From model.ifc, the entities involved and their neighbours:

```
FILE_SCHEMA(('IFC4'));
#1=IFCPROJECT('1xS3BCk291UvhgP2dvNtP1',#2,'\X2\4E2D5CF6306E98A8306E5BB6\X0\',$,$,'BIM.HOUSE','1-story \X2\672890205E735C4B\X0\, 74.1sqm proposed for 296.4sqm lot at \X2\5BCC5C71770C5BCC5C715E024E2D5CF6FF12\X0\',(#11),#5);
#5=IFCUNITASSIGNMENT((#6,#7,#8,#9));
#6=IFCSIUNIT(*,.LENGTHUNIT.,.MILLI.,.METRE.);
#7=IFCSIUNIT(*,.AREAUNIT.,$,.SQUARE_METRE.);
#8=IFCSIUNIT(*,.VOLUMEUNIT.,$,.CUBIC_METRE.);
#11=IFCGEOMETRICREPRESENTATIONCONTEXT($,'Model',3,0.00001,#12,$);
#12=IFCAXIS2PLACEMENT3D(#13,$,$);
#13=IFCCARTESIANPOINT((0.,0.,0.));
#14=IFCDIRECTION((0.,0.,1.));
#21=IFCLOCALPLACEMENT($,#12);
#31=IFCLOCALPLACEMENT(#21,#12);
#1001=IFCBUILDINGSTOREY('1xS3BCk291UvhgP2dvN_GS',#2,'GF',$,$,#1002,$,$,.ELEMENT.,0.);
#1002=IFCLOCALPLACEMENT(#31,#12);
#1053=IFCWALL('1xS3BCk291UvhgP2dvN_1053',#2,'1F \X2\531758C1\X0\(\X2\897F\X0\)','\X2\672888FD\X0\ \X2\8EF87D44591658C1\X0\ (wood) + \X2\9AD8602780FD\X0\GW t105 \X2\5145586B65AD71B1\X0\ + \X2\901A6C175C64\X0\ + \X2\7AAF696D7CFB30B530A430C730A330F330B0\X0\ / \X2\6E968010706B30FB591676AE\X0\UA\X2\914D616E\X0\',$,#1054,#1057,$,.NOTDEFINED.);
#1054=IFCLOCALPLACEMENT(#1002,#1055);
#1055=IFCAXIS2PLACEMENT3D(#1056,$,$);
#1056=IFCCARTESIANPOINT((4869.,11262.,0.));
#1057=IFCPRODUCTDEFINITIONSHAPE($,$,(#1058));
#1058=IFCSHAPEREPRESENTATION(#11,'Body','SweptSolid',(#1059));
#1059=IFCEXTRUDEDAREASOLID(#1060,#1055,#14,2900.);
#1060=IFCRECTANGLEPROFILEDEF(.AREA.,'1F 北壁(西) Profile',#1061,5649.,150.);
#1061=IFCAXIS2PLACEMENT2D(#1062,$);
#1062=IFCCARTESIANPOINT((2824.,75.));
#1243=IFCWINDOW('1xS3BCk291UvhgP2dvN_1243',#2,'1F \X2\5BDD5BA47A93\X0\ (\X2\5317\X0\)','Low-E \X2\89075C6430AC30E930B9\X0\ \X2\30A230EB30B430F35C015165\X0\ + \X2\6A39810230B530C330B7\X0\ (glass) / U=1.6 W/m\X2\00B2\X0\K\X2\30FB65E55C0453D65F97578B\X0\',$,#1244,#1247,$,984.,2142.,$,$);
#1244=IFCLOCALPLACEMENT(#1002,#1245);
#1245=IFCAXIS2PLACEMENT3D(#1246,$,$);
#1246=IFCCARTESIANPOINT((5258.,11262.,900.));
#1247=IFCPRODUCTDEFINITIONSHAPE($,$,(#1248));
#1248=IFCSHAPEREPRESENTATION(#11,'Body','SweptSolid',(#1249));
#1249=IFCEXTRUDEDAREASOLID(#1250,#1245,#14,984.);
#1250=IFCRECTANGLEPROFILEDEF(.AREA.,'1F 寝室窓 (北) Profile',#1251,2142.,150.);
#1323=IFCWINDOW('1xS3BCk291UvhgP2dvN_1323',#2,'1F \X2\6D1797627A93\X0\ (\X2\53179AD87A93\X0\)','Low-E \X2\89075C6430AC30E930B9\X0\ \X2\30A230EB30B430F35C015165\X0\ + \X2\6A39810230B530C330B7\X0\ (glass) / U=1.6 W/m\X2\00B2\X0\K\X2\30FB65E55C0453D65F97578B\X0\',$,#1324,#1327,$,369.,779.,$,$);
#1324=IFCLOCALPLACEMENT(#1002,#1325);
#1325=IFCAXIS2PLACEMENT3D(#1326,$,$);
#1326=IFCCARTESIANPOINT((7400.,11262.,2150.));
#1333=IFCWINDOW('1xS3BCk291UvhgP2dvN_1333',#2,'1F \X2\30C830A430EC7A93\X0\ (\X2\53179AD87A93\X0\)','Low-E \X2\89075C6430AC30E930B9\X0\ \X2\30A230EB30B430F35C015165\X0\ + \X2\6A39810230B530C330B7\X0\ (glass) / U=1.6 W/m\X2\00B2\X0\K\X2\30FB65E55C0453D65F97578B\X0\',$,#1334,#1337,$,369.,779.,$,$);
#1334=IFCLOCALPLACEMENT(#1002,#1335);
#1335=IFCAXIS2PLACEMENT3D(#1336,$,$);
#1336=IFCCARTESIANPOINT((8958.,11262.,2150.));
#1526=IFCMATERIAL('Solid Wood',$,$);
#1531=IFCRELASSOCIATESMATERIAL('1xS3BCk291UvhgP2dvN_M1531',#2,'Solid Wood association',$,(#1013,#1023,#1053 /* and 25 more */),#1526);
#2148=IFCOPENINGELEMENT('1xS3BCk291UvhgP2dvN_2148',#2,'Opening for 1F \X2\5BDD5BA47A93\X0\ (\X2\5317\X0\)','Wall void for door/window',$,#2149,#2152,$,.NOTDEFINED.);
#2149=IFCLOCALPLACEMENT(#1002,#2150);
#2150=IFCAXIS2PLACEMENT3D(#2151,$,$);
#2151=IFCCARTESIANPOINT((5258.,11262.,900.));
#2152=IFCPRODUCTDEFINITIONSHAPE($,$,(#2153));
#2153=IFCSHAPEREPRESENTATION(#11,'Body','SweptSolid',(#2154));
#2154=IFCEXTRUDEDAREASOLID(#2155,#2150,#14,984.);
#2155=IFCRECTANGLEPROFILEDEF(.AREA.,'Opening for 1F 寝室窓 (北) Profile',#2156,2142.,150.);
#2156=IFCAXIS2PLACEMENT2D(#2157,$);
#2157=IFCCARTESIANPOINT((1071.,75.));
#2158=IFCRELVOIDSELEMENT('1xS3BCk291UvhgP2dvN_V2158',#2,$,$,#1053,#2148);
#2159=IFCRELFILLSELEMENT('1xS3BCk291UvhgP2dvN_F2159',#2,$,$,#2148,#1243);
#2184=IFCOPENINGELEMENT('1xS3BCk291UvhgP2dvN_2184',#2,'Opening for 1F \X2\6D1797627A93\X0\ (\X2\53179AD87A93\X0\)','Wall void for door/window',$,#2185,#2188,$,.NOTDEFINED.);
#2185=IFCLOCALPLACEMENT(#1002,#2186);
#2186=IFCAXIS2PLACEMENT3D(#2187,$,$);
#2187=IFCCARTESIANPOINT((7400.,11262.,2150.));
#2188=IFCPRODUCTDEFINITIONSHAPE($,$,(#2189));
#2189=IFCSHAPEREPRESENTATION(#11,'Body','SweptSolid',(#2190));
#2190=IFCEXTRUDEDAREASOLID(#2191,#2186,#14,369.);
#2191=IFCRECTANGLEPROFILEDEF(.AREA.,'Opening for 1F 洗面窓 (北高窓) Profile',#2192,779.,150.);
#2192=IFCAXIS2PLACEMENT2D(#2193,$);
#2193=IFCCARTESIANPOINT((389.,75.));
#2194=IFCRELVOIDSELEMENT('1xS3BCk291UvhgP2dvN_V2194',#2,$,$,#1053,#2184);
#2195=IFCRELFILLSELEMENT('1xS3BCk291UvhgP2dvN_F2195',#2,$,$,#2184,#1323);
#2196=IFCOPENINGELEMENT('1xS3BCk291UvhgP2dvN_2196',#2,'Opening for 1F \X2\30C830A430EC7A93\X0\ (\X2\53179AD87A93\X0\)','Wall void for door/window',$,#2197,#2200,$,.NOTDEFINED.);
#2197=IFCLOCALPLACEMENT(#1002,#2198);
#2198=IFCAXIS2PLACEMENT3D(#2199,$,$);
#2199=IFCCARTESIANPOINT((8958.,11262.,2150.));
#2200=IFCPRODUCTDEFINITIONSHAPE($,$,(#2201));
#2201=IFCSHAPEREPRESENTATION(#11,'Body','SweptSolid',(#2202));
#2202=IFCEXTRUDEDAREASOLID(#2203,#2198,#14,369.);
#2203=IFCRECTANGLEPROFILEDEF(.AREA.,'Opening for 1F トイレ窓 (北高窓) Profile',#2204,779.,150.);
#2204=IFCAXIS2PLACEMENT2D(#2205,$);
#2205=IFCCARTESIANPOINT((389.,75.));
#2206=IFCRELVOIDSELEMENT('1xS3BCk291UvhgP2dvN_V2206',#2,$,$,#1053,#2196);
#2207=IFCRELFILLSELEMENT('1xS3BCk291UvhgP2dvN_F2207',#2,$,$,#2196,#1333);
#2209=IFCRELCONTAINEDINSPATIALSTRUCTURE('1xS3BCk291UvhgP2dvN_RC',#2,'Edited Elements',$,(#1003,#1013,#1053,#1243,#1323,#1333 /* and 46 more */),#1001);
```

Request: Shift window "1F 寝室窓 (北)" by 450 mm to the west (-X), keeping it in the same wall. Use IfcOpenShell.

```python
import ifcopenshell
import ifcopenshell.api.geometry
import ifcopenshell.util.placement

model = ifcopenshell.open("model.ifc")

window = model.by_guid("1xS3BCk291UvhgP2dvN_1243")
opening = window.FillsVoids[0].RelatingOpeningElement
wall = opening.VoidsElements[0].RelatingBuildingElement

wall_matrix = ifcopenshell.util.placement.get_local_placement(wall.ObjectPlacement)
shift = wall_matrix[:3, 0] * -450.0
before = ifcopenshell.util.placement.get_local_placement(window.ObjectPlacement)[:3, 3].copy()

# The window is not placed relative to its opening, so move both.
for product in (opening, window):
    matrix = ifcopenshell.util.placement.get_local_placement(product.ObjectPlacement)
    matrix[:3, 3] += shift
    ifcopenshell.api.geometry.edit_object_placement(model, product=product, matrix=matrix, is_si=False)

after = ifcopenshell.util.placement.get_local_placement(window.ObjectPlacement)[:3, 3]
print("window moved by", (after - before).round(3) + 0.0)

model.write("model_rev.ifc")
```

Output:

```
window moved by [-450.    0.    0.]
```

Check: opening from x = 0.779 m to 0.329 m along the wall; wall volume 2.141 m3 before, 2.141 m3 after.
